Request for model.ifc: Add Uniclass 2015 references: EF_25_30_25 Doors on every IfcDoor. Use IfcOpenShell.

First a look at what the model holds.

```python
import ifcopenshell

model = ifcopenshell.open("model.ifc")
print(model.schema)
print("classifications:", [c.Name for c in model.by_type("IfcClassification")])
for ifc_class in ("IfcDoor", "IfcRoof", "IfcStair", "IfcWall", "IfcWindow"):
    print(ifc_class, len(model.by_type(ifc_class)))
```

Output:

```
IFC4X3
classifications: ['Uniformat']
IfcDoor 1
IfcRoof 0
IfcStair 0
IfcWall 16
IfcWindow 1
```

```python
import ifcopenshell
import ifcopenshell.api.classification

model = ifcopenshell.open("model.ifc")

system = ifcopenshell.api.classification.add_classification(model, classification="Uniclass 2015")

codes = {
    "IfcDoor": ("EF_25_30_25", "Doors"),
}
for ifc_class, (code, name) in codes.items():
    products = model.by_type(ifc_class)
    ifcopenshell.api.classification.add_reference(
        model, products=products, classification=system, identification=code, name=name
    )
    print(code, len(products))

model.write("model-out.ifc")
```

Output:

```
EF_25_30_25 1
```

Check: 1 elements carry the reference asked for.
